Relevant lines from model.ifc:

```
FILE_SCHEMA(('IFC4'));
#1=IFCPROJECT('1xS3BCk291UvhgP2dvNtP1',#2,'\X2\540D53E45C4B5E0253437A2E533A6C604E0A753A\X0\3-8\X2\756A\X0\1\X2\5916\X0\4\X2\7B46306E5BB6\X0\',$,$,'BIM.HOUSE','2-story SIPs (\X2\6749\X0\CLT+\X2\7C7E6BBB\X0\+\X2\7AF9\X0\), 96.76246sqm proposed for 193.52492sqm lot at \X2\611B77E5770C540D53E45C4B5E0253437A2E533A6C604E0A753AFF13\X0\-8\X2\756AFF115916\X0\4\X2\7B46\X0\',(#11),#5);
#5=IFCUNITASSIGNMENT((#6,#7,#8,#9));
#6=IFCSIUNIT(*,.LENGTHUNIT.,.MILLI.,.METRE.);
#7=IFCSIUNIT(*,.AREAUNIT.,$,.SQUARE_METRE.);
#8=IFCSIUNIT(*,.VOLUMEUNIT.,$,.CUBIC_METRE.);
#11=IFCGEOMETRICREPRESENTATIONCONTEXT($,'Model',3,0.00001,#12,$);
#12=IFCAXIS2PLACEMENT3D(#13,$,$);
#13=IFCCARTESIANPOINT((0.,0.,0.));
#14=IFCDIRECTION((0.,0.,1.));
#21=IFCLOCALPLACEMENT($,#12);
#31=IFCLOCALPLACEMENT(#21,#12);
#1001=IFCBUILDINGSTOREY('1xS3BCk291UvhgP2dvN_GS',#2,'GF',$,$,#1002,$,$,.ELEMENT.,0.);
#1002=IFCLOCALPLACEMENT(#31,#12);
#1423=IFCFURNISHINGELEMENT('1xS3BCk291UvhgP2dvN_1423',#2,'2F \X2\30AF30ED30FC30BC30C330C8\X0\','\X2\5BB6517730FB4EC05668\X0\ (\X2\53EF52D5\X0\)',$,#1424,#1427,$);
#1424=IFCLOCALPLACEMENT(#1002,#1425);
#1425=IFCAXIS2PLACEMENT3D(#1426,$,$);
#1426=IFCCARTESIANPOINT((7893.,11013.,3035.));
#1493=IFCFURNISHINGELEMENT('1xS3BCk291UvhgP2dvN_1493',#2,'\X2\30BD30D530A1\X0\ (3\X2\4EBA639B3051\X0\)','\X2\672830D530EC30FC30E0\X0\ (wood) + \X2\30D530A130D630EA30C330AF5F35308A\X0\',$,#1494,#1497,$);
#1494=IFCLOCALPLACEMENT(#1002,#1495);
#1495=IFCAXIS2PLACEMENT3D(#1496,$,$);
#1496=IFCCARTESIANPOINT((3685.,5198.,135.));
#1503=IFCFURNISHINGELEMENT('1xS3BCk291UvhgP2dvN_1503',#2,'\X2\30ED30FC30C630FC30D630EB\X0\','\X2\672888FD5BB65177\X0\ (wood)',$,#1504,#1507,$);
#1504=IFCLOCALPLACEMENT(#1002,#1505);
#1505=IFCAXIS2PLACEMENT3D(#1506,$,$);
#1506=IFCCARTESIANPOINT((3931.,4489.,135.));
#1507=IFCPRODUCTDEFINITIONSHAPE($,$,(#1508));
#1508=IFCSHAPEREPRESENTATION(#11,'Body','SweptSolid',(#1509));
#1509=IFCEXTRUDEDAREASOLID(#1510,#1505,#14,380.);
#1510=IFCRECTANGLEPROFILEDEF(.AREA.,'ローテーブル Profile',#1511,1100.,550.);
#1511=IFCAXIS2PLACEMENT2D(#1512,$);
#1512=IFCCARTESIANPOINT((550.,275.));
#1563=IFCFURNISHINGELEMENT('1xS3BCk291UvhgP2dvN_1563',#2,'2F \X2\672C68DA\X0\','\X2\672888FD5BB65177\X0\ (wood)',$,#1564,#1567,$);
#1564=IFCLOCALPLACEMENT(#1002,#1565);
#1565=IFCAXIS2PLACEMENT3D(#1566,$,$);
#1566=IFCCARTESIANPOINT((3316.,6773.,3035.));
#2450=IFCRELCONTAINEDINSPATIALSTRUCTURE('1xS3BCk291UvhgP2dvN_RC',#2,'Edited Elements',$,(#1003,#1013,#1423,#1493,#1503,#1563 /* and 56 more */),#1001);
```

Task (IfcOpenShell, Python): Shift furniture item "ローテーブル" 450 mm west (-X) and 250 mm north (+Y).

```python
import ifcopenshell
import ifcopenshell.api.geometry
import ifcopenshell.util.placement
import ifcopenshell.util.unit

model = ifcopenshell.open("model.ifc")
unit_scale = ifcopenshell.util.unit.calculate_unit_scale(model)

item = model.by_guid("1xS3BCk291UvhgP2dvN_1503")
matrix = ifcopenshell.util.placement.get_local_placement(item.ObjectPlacement)
matrix[0, 3] -= 0.45 / unit_scale
matrix[1, 3] += 0.25 / unit_scale
ifcopenshell.api.geometry.edit_object_placement(model, product=item, matrix=matrix, is_si=False)

print(ifcopenshell.util.placement.get_local_placement(item.ObjectPlacement).round(3) + 0.0)

model.write("model-out.ifc")
```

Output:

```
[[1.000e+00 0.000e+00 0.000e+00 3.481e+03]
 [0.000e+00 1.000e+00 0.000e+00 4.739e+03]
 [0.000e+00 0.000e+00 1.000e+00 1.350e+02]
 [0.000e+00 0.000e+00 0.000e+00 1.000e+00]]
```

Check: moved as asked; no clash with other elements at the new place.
